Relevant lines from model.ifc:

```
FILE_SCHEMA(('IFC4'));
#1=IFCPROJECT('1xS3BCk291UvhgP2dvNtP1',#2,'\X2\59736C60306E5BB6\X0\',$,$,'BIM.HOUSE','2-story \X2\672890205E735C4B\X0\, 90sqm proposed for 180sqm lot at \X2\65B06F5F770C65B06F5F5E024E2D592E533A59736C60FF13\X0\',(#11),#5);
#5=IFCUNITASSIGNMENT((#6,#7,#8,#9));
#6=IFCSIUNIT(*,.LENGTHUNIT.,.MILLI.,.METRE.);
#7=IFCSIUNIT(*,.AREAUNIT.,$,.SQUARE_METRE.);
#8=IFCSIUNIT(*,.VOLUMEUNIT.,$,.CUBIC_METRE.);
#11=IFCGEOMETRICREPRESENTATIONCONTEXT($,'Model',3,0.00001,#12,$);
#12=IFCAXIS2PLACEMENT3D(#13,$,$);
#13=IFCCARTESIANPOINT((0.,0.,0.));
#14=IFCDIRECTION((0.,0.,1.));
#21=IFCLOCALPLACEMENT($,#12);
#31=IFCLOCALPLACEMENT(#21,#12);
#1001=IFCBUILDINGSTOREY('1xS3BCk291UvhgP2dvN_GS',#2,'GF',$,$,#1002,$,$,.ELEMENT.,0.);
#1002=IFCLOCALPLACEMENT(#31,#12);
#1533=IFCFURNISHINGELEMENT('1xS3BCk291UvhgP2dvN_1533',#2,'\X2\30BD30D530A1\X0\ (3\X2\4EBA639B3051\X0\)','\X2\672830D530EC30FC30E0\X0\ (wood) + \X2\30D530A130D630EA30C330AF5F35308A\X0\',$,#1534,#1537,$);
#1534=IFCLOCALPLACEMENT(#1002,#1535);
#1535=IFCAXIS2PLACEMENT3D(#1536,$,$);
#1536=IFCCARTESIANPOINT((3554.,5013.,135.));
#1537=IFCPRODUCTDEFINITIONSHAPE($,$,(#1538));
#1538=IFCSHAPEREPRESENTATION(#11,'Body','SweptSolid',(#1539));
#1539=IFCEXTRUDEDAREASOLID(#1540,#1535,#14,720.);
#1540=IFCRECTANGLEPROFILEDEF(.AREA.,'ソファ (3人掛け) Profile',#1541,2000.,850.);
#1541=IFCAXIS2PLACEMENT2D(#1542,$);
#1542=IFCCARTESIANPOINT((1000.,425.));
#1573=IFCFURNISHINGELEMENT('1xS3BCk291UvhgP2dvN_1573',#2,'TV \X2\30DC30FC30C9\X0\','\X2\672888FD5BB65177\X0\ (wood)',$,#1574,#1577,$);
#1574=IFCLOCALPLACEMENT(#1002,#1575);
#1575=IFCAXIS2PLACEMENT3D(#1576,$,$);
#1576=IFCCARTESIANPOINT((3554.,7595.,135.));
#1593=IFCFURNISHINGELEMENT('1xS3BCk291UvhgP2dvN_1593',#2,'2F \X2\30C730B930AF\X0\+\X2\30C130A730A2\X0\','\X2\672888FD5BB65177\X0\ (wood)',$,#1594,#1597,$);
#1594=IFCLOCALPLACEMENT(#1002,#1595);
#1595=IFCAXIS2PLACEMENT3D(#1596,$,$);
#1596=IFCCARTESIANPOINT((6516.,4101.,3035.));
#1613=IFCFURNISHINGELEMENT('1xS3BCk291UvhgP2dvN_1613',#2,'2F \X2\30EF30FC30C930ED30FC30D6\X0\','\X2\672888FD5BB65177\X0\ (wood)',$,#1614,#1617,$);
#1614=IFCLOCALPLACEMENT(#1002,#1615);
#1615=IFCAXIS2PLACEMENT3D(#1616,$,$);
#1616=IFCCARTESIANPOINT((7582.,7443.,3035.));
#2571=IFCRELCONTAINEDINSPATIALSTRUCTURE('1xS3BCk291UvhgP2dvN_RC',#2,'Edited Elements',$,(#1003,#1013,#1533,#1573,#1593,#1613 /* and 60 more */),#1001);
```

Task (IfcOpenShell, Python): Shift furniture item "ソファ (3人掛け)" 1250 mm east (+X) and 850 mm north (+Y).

```python
import ifcopenshell
import ifcopenshell.api.geometry
import ifcopenshell.util.placement
import ifcopenshell.util.unit

model = ifcopenshell.open("model.ifc")
unit_scale = ifcopenshell.util.unit.calculate_unit_scale(model)

item = model.by_guid("1xS3BCk291UvhgP2dvN_1533")
matrix = ifcopenshell.util.placement.get_local_placement(item.ObjectPlacement)
matrix[0, 3] += 1.25 / unit_scale
matrix[1, 3] += 0.85 / unit_scale
ifcopenshell.api.geometry.edit_object_placement(model, product=item, matrix=matrix, is_si=False)

print(ifcopenshell.util.placement.get_local_placement(item.ObjectPlacement).round(3) + 0.0)

model.write("model_edited.ifc")
```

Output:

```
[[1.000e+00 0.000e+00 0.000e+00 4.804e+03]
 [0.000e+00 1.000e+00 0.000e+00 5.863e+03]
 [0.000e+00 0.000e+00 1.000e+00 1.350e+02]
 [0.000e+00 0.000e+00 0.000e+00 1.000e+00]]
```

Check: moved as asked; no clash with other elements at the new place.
